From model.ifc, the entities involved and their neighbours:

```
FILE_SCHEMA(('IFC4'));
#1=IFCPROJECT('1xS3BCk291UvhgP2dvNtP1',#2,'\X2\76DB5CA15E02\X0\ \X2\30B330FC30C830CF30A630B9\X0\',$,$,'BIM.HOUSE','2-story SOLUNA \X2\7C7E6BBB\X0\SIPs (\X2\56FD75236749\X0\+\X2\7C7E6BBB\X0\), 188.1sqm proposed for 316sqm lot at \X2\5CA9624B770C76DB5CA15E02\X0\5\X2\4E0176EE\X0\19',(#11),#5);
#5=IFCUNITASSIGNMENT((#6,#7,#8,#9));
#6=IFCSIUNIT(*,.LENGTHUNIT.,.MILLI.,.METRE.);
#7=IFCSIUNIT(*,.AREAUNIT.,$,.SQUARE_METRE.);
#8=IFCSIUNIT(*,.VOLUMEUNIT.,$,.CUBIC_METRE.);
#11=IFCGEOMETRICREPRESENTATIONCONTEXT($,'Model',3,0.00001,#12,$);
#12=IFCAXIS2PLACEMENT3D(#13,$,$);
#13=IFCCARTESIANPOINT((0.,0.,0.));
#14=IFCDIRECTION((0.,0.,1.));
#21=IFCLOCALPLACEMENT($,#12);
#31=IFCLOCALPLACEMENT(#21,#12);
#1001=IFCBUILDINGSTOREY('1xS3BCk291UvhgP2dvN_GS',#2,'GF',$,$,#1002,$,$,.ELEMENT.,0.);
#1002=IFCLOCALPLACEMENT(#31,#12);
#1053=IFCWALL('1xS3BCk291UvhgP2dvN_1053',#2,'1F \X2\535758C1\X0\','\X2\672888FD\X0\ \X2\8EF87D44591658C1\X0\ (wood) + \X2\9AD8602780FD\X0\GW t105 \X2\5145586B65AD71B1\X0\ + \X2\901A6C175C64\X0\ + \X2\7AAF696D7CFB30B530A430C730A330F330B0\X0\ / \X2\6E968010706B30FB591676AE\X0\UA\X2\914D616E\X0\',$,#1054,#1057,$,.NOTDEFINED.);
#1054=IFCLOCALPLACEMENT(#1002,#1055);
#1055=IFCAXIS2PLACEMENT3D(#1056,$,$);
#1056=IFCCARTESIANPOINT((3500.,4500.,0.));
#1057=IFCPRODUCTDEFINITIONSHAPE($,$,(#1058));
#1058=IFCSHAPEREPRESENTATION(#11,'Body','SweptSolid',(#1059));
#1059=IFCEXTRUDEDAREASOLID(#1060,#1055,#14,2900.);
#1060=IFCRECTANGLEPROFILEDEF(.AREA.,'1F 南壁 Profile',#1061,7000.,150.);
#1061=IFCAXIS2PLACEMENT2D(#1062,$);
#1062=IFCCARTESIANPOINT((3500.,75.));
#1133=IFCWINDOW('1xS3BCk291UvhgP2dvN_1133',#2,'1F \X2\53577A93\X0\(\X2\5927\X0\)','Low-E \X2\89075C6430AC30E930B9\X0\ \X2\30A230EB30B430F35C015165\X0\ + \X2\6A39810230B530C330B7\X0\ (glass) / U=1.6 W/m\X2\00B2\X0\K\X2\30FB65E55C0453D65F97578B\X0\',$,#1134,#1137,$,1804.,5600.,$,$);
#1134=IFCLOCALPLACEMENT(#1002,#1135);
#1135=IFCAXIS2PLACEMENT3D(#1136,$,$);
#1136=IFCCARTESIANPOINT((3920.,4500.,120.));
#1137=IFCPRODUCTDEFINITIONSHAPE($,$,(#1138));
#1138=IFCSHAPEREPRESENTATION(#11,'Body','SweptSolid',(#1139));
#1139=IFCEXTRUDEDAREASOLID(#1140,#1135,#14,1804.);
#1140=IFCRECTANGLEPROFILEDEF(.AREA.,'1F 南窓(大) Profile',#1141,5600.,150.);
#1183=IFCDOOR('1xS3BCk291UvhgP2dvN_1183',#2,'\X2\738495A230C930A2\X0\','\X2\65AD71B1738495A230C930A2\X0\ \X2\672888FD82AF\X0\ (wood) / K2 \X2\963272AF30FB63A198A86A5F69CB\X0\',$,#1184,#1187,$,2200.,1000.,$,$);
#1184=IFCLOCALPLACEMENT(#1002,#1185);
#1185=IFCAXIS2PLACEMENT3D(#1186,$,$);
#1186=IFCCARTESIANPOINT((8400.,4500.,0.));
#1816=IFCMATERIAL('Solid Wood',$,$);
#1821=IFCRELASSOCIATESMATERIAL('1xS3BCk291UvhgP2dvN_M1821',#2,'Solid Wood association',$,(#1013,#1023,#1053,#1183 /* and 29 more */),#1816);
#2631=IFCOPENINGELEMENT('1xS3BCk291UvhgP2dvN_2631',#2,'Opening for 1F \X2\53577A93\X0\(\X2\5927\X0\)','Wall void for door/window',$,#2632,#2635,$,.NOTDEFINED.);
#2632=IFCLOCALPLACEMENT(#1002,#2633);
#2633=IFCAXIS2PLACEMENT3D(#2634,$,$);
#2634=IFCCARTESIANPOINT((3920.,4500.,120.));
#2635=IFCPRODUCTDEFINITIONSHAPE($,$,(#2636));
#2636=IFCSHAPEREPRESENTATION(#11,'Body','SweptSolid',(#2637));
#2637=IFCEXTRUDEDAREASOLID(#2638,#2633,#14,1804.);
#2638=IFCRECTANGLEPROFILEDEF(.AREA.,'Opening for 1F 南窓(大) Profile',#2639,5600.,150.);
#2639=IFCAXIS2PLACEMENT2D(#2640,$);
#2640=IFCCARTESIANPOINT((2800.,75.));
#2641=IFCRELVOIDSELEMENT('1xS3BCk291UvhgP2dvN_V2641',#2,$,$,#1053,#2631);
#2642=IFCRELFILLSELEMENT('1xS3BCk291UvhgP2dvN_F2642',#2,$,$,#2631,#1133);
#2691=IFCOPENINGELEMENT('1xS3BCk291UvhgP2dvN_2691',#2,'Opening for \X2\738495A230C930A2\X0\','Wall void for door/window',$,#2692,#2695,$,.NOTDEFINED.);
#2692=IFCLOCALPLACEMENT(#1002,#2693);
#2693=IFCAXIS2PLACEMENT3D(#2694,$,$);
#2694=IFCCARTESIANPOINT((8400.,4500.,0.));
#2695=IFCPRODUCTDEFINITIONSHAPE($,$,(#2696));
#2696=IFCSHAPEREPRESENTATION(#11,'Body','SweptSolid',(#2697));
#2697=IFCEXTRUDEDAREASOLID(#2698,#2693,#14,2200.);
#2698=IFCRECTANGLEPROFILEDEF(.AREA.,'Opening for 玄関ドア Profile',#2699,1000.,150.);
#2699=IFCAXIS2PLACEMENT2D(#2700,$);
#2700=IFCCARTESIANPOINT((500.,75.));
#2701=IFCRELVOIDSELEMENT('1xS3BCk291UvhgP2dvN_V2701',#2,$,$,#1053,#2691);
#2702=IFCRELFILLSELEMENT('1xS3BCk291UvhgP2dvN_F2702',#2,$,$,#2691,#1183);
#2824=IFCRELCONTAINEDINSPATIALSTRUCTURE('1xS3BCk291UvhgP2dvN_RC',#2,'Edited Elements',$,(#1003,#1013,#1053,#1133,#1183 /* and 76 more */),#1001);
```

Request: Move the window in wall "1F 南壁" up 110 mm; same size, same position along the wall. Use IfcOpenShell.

```python
import numpy as np
import ifcopenshell
import ifcopenshell.api.geometry
import ifcopenshell.util.placement
import ifcopenshell.util.unit

model = ifcopenshell.open("model.ifc")
unit_scale = ifcopenshell.util.unit.calculate_unit_scale(model)

window = model.by_guid("1xS3BCk291UvhgP2dvN_1133")
opening = window.FillsVoids[0].RelatingOpeningElement
dz = 0.11 / unit_scale

shift = np.array([0.0, 0.0, dz])
# The window is not placed relative to its opening, so move both.
for product in (opening, window):
    matrix = ifcopenshell.util.placement.get_local_placement(product.ObjectPlacement)
    matrix[:3, 3] += shift
    ifcopenshell.api.geometry.edit_object_placement(model, product=product, matrix=matrix, is_si=False)

print(f"moved by {dz * unit_scale:+.3f} m")

model.write("model_edited.ifc")
```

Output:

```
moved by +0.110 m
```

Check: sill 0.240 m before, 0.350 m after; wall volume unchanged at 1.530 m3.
